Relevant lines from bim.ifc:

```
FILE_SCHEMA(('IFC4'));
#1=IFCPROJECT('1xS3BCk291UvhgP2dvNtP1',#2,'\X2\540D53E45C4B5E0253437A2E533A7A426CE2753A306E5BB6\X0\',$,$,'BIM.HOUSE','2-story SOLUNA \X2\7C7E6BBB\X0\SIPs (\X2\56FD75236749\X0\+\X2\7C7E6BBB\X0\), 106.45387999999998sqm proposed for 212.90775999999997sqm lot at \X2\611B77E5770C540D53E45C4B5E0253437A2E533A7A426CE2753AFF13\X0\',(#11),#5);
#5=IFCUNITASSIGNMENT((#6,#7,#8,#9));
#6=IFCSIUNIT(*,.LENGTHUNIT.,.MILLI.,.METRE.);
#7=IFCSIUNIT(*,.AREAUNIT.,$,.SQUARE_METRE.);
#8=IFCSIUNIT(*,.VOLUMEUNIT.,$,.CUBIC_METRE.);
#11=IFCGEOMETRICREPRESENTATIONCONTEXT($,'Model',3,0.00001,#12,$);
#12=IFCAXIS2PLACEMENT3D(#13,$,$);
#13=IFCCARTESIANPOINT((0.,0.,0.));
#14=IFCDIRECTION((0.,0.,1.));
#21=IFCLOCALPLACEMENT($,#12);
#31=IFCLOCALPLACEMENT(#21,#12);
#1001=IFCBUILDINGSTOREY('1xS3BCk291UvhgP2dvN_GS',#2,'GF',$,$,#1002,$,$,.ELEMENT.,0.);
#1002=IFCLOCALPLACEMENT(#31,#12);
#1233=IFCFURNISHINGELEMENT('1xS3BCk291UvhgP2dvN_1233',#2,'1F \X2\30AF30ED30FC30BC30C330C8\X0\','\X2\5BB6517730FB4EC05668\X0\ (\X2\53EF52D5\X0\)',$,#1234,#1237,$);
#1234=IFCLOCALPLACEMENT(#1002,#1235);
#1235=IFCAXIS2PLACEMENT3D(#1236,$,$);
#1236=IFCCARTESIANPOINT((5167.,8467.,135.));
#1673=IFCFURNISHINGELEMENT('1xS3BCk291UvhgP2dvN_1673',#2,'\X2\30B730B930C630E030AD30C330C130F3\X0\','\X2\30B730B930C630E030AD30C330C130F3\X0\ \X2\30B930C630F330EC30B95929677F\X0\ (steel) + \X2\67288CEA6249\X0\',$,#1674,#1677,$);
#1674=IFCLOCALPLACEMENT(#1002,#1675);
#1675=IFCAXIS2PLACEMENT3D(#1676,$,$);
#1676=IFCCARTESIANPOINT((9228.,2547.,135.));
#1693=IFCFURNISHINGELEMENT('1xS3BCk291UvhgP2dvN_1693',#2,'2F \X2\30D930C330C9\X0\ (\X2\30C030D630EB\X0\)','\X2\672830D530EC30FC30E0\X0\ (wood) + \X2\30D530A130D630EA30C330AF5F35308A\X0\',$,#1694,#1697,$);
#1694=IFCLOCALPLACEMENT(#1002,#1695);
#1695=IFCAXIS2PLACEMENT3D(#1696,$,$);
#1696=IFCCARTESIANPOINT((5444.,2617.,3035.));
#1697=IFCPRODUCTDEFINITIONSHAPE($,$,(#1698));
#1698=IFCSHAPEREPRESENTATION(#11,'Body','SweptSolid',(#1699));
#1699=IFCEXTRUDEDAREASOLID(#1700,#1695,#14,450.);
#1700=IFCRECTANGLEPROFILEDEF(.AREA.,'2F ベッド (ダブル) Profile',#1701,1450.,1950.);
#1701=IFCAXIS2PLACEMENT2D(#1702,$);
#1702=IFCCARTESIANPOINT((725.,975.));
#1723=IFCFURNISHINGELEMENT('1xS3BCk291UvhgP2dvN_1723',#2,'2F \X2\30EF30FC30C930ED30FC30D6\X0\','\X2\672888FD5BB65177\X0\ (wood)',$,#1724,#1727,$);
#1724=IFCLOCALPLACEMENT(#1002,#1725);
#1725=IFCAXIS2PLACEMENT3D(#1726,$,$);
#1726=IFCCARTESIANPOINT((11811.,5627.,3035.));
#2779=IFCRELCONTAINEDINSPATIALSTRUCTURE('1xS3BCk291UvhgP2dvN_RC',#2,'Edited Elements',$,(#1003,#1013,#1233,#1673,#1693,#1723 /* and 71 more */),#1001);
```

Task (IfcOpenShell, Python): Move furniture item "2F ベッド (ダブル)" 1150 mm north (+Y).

```python
import ifcopenshell
import ifcopenshell.api.geometry
import ifcopenshell.util.placement
import ifcopenshell.util.unit

model = ifcopenshell.open("bim.ifc")
unit_scale = ifcopenshell.util.unit.calculate_unit_scale(model)

item = model.by_guid("1xS3BCk291UvhgP2dvN_1693")
matrix = ifcopenshell.util.placement.get_local_placement(item.ObjectPlacement)
matrix[1, 3] += 1.15 / unit_scale
ifcopenshell.api.geometry.edit_object_placement(model, product=item, matrix=matrix, is_si=False)

print(ifcopenshell.util.placement.get_local_placement(item.ObjectPlacement).round(3) + 0.0)

model.write("bim_rev.ifc")
```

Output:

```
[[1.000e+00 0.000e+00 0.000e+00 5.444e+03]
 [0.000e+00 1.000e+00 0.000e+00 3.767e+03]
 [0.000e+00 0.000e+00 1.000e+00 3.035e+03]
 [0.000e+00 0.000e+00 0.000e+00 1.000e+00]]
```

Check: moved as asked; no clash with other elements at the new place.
